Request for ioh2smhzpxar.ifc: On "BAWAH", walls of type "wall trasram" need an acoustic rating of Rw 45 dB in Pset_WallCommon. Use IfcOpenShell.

First a look at what the model holds.

```python
import ifcopenshell
import ifcopenshell.util.element

model = ifcopenshell.open("ioh2smhzpxar.ifc")
print(model.schema)
storey = next(s for s in model.by_type("IfcBuildingStorey") if s.Name == "BAWAH")
walls = [e for e in ifcopenshell.util.element.get_decomposition(storey) if e.is_a("IfcWall")]
seen = {}
for e in walls:
    element_type = ifcopenshell.util.element.get_type(e)
    key = (element_type.Name if element_type != e and element_type else None, ifcopenshell.util.element.get_pset(e, "Pset_WallCommon", "AcousticRating"))
    seen[key] = seen.get(key, 0) + 1
for (name, value), count in sorted(seen.items(), key=str):
    print(count, "x", name, "|", value)
```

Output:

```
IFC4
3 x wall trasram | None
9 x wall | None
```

```python
import ifcopenshell
import ifcopenshell.api.pset
import ifcopenshell.util.element

model = ifcopenshell.open("ioh2smhzpxar.ifc")

storey = next(s for s in model.by_type("IfcBuildingStorey") if s.Name == "BAWAH")
walls = [e for e in ifcopenshell.util.element.get_decomposition(storey) if e.is_a("IfcWall")]

count = 0
for e in walls:
    element_type = ifcopenshell.util.element.get_type(e)
    if element_type in (None, e) or element_type.Name != "wall trasram":
        continue
    # add_pset returns the element's existing set when there is one.
    pset = ifcopenshell.api.pset.add_pset(model, product=e, name="Pset_WallCommon")
    ifcopenshell.api.pset.edit_pset(model, pset=pset, properties={"AcousticRating": "Rw 45 dB"})
    count += 1

print(count, "walls updated")

model.write("ioh2smhzpxar_updated.ifc")
```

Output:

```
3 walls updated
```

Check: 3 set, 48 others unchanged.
